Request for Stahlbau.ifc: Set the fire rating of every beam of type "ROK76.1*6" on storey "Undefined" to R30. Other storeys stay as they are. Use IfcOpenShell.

First a look at what the model holds.

```python
import ifcopenshell
import ifcopenshell.util.element

model = ifcopenshell.open("Stahlbau.ifc")
print(model.schema)
storey = next(s for s in model.by_type("IfcBuildingStorey") if s.Name == "Undefined")
beams = [e for e in ifcopenshell.util.element.get_decomposition(storey) if e.is_a("IfcBeam")]
seen = {}
for e in beams:
    element_type = ifcopenshell.util.element.get_type(e)
    key = (element_type.Name if element_type != e and element_type else None, ifcopenshell.util.element.get_pset(e, "Pset_BeamCommon", "FireRating"))
    seen[key] = seen.get(key, 0) + 1
for (name, value), count in sorted(seen.items(), key=str):
    print(count, "x", name, "|", value)
```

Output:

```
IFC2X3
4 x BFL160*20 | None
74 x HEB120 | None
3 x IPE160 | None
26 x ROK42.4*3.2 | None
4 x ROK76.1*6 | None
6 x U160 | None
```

```python
import ifcopenshell
import ifcopenshell.api.pset
import ifcopenshell.util.element

model = ifcopenshell.open("Stahlbau.ifc")

storey = next(s for s in model.by_type("IfcBuildingStorey") if s.Name == "Undefined")
beams = [e for e in ifcopenshell.util.element.get_decomposition(storey) if e.is_a("IfcBeam")]

count = 0
for e in beams:
    element_type = ifcopenshell.util.element.get_type(e)
    if element_type in (None, e) or element_type.Name != "ROK76.1*6":
        continue
    # add_pset returns the element's existing set when there is one.
    pset = ifcopenshell.api.pset.add_pset(model, product=e, name="Pset_BeamCommon")
    ifcopenshell.api.pset.edit_pset(model, pset=pset, properties={"FireRating": "R30"})
    count += 1

print(count, "beams updated")

model.write("Stahlbau_v2.ifc")
```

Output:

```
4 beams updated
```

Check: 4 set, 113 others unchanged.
